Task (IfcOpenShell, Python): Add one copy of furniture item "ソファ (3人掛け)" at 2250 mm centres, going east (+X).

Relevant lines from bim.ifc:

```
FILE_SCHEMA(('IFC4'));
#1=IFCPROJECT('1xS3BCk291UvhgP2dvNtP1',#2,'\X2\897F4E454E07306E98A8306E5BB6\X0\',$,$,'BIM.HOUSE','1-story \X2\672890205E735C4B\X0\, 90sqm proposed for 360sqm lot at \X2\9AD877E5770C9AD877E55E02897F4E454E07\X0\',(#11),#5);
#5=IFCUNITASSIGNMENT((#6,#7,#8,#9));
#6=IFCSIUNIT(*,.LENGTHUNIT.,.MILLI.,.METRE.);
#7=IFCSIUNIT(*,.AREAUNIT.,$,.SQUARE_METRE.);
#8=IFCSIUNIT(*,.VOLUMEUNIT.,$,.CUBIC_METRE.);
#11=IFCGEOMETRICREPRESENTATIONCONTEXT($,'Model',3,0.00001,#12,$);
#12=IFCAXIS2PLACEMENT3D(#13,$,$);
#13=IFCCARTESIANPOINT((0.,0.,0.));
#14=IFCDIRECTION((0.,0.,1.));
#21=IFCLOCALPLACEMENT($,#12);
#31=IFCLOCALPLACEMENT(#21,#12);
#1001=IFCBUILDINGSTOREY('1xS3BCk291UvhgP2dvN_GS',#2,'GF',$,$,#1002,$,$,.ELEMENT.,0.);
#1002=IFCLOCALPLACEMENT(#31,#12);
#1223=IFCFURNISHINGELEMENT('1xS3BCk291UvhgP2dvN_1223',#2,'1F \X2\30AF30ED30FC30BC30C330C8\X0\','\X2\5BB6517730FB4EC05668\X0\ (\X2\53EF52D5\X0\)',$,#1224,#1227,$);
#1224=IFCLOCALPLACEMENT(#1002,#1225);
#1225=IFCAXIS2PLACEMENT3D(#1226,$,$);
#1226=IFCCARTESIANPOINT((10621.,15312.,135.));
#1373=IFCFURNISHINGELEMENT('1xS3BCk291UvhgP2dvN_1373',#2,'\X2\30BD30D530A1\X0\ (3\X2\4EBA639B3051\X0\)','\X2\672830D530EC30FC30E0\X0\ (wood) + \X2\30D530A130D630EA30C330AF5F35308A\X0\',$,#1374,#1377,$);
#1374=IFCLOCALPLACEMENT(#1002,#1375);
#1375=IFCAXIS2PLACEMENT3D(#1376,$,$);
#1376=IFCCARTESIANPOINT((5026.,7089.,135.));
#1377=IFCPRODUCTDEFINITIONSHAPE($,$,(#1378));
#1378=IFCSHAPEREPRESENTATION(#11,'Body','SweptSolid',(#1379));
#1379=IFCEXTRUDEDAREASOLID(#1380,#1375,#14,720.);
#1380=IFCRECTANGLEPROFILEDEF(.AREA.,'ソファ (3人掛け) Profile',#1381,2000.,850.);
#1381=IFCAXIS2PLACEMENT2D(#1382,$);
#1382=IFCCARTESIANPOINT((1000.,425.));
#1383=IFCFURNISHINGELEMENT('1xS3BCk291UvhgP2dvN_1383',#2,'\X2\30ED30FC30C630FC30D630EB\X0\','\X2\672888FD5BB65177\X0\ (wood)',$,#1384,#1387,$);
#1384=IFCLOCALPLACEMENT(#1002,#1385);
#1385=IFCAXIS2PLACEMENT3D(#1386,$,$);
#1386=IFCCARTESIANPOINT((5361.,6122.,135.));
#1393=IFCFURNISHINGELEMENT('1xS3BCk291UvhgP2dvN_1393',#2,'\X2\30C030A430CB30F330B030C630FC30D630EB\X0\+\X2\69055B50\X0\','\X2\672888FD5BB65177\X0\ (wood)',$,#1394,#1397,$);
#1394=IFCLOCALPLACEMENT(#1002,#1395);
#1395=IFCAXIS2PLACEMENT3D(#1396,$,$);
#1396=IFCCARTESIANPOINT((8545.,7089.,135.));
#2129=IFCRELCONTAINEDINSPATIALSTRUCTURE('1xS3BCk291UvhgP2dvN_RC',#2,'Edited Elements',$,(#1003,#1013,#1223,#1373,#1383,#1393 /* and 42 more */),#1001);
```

```python
import numpy as np
import ifcopenshell
import ifcopenshell.api.geometry
import ifcopenshell.api.root
import ifcopenshell.util.element
import ifcopenshell.util.placement

model = ifcopenshell.open("bim.ifc")


def reuse_history(source, copy):
    """copy_class also copies each property set's owner history, people and application; keep the originals."""
    for rel in copy.IsDefinedBy:
        if rel.is_a("IfcRelDefinesByProperties") and (history := rel.RelatingPropertyDefinition.OwnerHistory):
            rel.RelatingPropertyDefinition.OwnerHistory = source.OwnerHistory
            ifcopenshell.util.element.remove_deep2(model, history)


source = model.by_id(1373)
base = ifcopenshell.util.placement.get_local_placement(source.ObjectPlacement)
step = np.array([1.0, 0.0, 0.0]) * 2250.0

for i in range(1, 2):
    copy = ifcopenshell.api.root.copy_class(model, product=source)
    copy.Representation = ifcopenshell.util.element.copy_deep(
        model, source.Representation, exclude=["IfcGeometricRepresentationContext", "IfcRepresentationMap"]
    )
    reuse_history(source, copy)
    matrix = base.copy()
    matrix[:3, 3] += i * step
    print("added at", matrix[:3, 3].round(3) + 0.0)
    ifcopenshell.api.geometry.edit_object_placement(model, product=copy, matrix=matrix, is_si=False)

model.write("bim-out.ifc")
```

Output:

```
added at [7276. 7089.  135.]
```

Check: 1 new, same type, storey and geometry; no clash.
